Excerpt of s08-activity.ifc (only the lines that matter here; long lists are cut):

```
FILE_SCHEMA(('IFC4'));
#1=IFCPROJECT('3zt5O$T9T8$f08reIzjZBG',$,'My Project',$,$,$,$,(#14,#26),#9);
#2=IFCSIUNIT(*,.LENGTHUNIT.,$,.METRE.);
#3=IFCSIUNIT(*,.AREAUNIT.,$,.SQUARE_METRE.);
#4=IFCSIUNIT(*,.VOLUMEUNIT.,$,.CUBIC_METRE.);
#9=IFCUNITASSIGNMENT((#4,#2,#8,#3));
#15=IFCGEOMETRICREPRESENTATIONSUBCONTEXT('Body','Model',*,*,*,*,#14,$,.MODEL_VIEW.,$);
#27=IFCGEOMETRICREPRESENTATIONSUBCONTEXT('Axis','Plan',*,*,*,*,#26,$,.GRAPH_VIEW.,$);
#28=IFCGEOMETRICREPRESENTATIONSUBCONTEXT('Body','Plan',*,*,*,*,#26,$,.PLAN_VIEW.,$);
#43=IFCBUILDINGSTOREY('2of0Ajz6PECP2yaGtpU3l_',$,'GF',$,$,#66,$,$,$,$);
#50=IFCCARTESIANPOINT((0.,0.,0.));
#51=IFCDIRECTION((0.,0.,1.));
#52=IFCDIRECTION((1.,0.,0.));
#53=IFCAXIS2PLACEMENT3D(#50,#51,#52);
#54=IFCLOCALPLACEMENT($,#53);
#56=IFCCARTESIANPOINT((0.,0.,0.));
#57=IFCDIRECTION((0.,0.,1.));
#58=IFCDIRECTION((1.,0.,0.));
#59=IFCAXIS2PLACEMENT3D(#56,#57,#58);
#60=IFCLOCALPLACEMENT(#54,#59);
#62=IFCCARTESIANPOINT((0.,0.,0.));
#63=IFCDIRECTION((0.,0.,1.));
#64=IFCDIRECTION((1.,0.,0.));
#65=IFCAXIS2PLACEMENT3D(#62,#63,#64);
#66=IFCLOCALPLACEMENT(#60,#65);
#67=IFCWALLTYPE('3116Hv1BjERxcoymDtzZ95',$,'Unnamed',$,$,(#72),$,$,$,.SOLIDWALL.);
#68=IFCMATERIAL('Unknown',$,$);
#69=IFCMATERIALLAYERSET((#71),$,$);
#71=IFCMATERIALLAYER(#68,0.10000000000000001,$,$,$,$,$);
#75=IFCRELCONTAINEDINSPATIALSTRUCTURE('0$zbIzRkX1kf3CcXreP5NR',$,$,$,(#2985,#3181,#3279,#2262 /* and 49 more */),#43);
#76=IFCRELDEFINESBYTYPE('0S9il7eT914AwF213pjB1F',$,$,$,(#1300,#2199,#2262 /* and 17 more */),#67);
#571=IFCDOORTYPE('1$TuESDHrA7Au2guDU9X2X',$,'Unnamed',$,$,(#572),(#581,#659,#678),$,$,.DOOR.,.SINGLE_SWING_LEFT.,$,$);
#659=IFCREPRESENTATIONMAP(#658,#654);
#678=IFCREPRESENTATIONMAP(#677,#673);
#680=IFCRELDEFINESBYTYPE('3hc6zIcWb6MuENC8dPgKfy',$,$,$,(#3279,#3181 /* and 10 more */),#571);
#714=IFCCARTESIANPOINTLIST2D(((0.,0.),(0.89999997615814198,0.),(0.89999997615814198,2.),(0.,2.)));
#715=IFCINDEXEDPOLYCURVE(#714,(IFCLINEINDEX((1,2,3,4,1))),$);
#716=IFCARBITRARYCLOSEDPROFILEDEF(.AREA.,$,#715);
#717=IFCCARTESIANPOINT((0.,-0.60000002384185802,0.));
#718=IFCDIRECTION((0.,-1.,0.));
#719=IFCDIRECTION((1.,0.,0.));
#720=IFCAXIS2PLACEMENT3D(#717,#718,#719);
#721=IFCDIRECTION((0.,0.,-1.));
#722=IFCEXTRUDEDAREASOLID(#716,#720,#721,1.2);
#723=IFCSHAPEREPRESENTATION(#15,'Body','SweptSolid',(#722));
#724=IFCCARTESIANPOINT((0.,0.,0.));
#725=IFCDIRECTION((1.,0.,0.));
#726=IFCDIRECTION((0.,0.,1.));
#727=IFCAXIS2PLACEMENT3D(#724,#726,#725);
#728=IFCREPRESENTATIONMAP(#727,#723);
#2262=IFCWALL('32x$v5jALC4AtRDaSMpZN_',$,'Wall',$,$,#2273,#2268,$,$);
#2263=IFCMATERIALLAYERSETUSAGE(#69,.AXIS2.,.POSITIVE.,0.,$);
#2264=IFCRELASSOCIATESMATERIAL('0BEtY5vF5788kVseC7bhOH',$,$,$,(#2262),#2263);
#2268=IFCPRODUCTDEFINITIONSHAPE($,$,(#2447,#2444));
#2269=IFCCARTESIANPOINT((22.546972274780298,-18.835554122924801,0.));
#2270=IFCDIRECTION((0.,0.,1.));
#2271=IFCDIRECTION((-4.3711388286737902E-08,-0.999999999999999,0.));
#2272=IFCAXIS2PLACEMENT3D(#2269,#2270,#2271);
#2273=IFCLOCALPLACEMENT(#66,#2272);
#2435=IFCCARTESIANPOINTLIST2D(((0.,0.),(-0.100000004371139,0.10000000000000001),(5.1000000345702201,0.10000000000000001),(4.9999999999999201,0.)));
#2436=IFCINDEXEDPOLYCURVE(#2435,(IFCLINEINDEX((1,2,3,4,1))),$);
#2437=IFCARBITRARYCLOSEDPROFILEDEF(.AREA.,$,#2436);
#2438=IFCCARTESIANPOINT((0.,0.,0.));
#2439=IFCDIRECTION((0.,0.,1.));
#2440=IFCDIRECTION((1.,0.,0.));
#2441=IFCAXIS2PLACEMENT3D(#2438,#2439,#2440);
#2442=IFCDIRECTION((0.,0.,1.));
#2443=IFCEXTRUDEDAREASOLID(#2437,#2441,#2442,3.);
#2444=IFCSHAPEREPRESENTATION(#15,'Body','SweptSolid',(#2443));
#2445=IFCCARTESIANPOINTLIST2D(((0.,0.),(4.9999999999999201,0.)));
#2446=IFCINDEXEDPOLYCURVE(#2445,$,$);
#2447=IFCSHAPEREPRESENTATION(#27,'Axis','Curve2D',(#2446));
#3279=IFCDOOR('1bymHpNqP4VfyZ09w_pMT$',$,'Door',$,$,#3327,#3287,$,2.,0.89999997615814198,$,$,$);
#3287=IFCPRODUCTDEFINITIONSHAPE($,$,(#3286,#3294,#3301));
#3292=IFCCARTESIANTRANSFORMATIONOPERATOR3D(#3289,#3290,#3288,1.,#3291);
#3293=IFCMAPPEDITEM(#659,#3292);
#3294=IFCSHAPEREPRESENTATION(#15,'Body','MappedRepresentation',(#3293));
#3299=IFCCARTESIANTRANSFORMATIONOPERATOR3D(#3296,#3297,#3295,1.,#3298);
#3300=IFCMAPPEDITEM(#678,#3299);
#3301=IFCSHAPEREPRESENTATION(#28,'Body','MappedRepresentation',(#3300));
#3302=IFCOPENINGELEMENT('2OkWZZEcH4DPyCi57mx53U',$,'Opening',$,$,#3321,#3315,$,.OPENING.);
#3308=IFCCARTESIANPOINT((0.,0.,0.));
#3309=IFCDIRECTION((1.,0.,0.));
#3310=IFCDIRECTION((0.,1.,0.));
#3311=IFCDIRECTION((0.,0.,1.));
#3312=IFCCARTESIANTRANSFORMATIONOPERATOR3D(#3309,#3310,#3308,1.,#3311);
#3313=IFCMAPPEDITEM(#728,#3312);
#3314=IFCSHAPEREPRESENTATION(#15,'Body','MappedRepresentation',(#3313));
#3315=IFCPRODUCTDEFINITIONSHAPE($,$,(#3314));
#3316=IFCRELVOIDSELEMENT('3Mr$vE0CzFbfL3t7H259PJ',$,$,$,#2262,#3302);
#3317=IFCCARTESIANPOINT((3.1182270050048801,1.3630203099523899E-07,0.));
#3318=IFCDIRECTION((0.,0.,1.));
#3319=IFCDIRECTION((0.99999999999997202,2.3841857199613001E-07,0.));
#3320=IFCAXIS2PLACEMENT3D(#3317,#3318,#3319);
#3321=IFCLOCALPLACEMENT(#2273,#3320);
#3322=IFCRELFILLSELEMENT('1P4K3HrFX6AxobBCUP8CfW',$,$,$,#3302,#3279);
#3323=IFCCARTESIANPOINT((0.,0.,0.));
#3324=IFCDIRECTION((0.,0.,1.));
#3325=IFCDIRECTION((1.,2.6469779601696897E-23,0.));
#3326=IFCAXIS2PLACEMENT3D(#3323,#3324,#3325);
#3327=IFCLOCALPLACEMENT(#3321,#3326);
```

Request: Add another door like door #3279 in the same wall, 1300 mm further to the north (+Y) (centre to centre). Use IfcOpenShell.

```python
import ifcopenshell
import ifcopenshell.api.feature
import ifcopenshell.api.geometry
import ifcopenshell.api.root
import ifcopenshell.geom
import ifcopenshell.util.element
import ifcopenshell.util.placement
import ifcopenshell.util.shape
import ifcopenshell.util.unit

model = ifcopenshell.open("s08-activity.ifc")
unit_scale = ifcopenshell.util.unit.calculate_unit_scale(model)
settings = ifcopenshell.geom.settings()


def volume(element):
    """Net volume in cubic metres, openings subtracted."""
    shape = ifcopenshell.geom.create_shape(settings, element)
    return ifcopenshell.util.shape.get_volume(shape.geometry)


door = model.by_id(3279)
opening = door.FillsVoids[0].RelatingOpeningElement
wall = opening.VoidsElements[0].RelatingBuildingElement
before = volume(wall)
shift = ifcopenshell.util.placement.get_local_placement(wall.ObjectPlacement)[:3, 0] * -1.3 / unit_scale

# copy_class copies the void relationship, type, container and properties, but no geometry.
new_opening = ifcopenshell.api.root.copy_class(model, product=opening)
new_opening.Representation = ifcopenshell.util.element.copy_deep(
    model, opening.Representation, exclude=["IfcGeometricRepresentationContext", "IfcRepresentationMap"]
)
new_door = ifcopenshell.api.root.copy_class(model, product=door)
new_door.Representation = ifcopenshell.util.element.copy_deep(
    model, door.Representation, exclude=["IfcGeometricRepresentationContext", "IfcRepresentationMap"]
)
ifcopenshell.api.feature.add_filling(model, opening=new_opening, element=new_door)

for old, new in ((opening, new_opening), (door, new_door)):
    matrix = ifcopenshell.util.placement.get_local_placement(old.ObjectPlacement)
    matrix[:3, 3] += shift
    ifcopenshell.api.geometry.edit_object_placement(model, product=new, matrix=matrix, is_si=False)

after = volume(wall)

print(f"wall volume {before:.3f} -> {after:.3f} m3")

model.write("s08-activity_v2.ifc")
```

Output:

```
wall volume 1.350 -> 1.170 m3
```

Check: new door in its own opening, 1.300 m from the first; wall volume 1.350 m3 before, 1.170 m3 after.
